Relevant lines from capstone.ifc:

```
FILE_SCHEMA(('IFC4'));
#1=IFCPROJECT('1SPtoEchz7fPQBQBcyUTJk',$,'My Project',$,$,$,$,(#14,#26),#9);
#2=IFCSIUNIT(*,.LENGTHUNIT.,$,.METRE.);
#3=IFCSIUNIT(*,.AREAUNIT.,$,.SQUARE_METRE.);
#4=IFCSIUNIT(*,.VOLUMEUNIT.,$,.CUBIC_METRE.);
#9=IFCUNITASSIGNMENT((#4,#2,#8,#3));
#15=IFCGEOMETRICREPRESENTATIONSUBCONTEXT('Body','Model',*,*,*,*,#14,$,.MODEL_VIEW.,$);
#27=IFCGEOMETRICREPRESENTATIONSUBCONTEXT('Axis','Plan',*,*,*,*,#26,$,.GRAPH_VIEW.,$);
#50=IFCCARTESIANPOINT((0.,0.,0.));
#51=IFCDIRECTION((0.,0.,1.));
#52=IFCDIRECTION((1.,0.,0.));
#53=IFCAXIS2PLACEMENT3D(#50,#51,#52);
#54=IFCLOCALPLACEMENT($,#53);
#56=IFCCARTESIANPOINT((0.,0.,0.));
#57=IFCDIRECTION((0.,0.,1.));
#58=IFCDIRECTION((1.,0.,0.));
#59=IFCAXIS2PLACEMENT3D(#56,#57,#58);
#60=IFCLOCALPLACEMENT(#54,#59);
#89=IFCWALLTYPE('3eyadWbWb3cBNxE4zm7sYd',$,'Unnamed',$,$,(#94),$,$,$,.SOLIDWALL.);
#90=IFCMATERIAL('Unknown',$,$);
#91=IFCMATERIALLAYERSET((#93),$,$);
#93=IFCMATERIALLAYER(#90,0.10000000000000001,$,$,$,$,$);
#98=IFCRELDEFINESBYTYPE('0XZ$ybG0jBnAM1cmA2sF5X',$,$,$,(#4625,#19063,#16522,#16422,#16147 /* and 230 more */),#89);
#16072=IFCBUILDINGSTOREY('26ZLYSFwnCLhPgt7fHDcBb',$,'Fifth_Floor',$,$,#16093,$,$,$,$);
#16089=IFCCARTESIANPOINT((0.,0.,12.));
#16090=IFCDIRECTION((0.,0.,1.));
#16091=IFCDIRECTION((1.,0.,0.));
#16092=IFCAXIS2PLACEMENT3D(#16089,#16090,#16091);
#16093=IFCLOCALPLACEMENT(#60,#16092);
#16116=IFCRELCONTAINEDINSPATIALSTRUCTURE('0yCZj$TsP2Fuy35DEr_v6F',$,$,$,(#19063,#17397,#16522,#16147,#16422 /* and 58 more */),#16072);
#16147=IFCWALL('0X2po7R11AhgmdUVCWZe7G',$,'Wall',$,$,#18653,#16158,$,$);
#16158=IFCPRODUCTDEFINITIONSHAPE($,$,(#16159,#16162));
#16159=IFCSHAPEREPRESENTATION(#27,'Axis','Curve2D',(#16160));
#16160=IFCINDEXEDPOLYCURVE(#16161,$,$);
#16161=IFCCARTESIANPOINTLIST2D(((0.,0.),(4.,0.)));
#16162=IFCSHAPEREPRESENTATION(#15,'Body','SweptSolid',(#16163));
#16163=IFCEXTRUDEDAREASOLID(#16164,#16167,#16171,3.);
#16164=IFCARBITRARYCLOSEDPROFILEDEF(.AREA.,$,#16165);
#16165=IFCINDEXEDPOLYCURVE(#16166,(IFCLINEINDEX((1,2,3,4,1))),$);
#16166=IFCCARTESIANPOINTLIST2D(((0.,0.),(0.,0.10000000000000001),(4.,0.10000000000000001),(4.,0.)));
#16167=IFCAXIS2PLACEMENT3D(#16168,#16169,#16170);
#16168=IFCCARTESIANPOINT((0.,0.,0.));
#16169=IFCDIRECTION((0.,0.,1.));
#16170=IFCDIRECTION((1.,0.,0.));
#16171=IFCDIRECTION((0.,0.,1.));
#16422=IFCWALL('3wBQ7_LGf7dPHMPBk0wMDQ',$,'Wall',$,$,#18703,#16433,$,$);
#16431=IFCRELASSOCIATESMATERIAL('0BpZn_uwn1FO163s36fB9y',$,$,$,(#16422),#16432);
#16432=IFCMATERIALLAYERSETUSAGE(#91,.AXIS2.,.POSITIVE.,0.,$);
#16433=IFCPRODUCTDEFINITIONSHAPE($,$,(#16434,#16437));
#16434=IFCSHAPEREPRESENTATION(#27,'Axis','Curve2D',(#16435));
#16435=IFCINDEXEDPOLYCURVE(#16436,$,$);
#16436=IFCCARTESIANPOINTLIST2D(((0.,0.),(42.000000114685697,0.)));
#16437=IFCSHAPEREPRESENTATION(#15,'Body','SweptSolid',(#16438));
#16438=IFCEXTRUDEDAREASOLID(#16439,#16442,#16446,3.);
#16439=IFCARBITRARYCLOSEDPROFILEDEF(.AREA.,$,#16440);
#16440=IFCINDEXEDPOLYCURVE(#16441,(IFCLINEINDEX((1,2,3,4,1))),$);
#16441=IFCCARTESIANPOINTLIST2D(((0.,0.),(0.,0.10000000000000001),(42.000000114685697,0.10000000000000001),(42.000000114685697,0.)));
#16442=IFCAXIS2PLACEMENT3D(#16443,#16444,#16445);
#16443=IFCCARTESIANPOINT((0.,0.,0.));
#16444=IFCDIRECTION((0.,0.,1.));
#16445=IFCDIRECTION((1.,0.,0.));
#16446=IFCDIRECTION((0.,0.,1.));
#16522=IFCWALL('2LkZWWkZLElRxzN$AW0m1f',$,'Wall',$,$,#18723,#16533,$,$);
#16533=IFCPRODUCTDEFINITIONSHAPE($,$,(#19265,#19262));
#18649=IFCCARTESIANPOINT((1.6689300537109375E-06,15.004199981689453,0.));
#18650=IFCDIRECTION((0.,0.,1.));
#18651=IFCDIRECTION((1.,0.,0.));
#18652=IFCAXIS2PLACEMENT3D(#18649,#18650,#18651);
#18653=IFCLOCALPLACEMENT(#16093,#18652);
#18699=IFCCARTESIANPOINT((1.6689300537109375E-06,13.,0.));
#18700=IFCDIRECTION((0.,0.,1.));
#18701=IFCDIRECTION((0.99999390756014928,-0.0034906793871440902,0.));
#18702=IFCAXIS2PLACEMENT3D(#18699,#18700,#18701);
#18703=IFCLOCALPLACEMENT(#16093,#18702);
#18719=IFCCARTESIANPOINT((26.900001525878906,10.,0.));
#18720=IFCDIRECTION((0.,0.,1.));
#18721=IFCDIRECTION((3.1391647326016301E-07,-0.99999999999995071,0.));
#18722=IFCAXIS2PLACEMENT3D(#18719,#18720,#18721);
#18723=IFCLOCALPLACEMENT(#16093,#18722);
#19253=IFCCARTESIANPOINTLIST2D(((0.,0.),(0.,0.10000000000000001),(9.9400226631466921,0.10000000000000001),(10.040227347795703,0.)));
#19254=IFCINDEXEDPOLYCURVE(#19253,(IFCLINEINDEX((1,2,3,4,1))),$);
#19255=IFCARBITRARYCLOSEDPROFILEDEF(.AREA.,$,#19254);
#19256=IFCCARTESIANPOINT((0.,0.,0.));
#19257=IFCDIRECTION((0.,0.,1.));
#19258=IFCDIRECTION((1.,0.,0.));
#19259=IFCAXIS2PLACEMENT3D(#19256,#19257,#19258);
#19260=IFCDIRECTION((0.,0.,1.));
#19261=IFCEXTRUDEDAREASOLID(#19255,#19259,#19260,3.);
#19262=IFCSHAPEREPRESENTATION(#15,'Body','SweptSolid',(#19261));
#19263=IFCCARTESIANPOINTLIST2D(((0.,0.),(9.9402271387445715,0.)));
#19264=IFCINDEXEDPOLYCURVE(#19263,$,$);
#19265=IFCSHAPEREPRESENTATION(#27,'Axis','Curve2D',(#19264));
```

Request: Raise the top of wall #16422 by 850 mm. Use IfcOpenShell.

```python
import ifcopenshell
import ifcopenshell.geom
import ifcopenshell.util.representation
import ifcopenshell.util.shape

model = ifcopenshell.open("capstone.ifc")
settings = ifcopenshell.geom.settings()


def volume(element):
    """Net volume in cubic metres, openings subtracted."""
    shape = ifcopenshell.geom.create_shape(settings, element)
    return ifcopenshell.util.shape.get_volume(shape.geometry)


wall = model.by_guid("3wBQ7_LGf7dPHMPBk0wMDQ")
before = volume(wall)

body = ifcopenshell.util.representation.get_representation(wall, "Model", "Body")
solid = body.Items[0]
old_height = solid.Depth
solid.Depth += 0.85
after = volume(wall)

print(f"height {old_height:g} -> {solid.Depth:g}, volume {before:.3f} -> {after:.3f} m3")

model.write("capstone_rev.ifc")
```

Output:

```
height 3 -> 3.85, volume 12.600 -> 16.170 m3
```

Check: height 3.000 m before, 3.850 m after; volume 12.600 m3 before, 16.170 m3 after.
